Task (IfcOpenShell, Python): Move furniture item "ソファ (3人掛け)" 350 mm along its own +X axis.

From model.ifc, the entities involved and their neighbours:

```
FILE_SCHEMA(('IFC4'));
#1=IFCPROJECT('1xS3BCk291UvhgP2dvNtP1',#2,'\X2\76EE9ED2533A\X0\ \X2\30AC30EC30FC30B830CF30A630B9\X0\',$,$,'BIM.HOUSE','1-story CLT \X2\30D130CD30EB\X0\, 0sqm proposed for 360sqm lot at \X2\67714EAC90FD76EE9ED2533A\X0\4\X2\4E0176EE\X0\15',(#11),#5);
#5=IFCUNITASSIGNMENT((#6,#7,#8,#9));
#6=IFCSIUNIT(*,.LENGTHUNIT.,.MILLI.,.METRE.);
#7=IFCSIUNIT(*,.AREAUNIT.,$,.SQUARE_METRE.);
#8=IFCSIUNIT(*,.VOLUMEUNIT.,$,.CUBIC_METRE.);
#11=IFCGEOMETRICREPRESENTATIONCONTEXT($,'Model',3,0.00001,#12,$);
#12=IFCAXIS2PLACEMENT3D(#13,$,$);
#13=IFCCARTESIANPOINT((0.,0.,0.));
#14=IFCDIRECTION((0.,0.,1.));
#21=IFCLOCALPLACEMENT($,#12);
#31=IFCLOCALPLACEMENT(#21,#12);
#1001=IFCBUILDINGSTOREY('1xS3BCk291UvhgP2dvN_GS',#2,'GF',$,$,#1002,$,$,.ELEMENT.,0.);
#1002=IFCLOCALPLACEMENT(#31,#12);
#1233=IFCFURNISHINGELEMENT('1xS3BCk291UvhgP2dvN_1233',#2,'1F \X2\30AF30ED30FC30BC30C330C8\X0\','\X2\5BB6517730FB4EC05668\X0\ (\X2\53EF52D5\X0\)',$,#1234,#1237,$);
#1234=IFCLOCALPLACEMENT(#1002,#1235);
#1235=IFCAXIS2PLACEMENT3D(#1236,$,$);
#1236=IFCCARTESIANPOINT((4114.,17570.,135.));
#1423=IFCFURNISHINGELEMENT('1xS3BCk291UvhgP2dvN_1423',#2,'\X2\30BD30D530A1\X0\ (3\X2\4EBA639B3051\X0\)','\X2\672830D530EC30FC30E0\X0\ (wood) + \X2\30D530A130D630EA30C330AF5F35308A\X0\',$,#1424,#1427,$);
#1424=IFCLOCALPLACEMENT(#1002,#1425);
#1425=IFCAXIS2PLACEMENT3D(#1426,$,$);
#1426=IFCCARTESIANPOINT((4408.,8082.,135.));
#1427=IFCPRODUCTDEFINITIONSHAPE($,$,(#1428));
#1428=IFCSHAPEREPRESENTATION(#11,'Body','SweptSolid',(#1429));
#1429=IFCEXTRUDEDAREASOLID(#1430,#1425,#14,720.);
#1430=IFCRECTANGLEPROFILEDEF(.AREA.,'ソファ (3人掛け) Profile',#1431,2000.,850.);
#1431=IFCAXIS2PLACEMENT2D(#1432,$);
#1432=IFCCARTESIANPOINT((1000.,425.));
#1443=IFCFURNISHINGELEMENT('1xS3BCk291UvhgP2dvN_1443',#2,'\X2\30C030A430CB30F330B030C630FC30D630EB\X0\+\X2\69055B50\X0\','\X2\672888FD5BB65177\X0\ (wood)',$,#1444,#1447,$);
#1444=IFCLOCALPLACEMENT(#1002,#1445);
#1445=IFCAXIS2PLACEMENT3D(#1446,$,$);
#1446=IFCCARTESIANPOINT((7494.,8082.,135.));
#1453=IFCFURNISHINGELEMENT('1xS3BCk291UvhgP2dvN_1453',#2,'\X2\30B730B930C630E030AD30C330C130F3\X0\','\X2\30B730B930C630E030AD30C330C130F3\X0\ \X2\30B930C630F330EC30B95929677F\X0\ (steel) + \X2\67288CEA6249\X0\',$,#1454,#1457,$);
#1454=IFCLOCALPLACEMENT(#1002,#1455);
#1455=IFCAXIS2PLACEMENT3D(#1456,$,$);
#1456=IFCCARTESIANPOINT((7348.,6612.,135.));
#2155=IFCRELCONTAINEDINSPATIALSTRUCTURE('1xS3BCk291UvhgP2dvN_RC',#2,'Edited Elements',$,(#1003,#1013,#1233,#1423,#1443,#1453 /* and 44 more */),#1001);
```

```python
import ifcopenshell
import ifcopenshell.api.geometry
import ifcopenshell.util.placement

model = ifcopenshell.open("model.ifc")

item = model.by_guid("1xS3BCk291UvhgP2dvN_1423")
matrix = ifcopenshell.util.placement.get_local_placement(item.ObjectPlacement)
matrix[:3, 3] += matrix[:3, 0] * 350.0
ifcopenshell.api.geometry.edit_object_placement(model, product=item, matrix=matrix, is_si=False)

print(ifcopenshell.util.placement.get_local_placement(item.ObjectPlacement).round(3) + 0.0)

model.write("model_v2.ifc")
```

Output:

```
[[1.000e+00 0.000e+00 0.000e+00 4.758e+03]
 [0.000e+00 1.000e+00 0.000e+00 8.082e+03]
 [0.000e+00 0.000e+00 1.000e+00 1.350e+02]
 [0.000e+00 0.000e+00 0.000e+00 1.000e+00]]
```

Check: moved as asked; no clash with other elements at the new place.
